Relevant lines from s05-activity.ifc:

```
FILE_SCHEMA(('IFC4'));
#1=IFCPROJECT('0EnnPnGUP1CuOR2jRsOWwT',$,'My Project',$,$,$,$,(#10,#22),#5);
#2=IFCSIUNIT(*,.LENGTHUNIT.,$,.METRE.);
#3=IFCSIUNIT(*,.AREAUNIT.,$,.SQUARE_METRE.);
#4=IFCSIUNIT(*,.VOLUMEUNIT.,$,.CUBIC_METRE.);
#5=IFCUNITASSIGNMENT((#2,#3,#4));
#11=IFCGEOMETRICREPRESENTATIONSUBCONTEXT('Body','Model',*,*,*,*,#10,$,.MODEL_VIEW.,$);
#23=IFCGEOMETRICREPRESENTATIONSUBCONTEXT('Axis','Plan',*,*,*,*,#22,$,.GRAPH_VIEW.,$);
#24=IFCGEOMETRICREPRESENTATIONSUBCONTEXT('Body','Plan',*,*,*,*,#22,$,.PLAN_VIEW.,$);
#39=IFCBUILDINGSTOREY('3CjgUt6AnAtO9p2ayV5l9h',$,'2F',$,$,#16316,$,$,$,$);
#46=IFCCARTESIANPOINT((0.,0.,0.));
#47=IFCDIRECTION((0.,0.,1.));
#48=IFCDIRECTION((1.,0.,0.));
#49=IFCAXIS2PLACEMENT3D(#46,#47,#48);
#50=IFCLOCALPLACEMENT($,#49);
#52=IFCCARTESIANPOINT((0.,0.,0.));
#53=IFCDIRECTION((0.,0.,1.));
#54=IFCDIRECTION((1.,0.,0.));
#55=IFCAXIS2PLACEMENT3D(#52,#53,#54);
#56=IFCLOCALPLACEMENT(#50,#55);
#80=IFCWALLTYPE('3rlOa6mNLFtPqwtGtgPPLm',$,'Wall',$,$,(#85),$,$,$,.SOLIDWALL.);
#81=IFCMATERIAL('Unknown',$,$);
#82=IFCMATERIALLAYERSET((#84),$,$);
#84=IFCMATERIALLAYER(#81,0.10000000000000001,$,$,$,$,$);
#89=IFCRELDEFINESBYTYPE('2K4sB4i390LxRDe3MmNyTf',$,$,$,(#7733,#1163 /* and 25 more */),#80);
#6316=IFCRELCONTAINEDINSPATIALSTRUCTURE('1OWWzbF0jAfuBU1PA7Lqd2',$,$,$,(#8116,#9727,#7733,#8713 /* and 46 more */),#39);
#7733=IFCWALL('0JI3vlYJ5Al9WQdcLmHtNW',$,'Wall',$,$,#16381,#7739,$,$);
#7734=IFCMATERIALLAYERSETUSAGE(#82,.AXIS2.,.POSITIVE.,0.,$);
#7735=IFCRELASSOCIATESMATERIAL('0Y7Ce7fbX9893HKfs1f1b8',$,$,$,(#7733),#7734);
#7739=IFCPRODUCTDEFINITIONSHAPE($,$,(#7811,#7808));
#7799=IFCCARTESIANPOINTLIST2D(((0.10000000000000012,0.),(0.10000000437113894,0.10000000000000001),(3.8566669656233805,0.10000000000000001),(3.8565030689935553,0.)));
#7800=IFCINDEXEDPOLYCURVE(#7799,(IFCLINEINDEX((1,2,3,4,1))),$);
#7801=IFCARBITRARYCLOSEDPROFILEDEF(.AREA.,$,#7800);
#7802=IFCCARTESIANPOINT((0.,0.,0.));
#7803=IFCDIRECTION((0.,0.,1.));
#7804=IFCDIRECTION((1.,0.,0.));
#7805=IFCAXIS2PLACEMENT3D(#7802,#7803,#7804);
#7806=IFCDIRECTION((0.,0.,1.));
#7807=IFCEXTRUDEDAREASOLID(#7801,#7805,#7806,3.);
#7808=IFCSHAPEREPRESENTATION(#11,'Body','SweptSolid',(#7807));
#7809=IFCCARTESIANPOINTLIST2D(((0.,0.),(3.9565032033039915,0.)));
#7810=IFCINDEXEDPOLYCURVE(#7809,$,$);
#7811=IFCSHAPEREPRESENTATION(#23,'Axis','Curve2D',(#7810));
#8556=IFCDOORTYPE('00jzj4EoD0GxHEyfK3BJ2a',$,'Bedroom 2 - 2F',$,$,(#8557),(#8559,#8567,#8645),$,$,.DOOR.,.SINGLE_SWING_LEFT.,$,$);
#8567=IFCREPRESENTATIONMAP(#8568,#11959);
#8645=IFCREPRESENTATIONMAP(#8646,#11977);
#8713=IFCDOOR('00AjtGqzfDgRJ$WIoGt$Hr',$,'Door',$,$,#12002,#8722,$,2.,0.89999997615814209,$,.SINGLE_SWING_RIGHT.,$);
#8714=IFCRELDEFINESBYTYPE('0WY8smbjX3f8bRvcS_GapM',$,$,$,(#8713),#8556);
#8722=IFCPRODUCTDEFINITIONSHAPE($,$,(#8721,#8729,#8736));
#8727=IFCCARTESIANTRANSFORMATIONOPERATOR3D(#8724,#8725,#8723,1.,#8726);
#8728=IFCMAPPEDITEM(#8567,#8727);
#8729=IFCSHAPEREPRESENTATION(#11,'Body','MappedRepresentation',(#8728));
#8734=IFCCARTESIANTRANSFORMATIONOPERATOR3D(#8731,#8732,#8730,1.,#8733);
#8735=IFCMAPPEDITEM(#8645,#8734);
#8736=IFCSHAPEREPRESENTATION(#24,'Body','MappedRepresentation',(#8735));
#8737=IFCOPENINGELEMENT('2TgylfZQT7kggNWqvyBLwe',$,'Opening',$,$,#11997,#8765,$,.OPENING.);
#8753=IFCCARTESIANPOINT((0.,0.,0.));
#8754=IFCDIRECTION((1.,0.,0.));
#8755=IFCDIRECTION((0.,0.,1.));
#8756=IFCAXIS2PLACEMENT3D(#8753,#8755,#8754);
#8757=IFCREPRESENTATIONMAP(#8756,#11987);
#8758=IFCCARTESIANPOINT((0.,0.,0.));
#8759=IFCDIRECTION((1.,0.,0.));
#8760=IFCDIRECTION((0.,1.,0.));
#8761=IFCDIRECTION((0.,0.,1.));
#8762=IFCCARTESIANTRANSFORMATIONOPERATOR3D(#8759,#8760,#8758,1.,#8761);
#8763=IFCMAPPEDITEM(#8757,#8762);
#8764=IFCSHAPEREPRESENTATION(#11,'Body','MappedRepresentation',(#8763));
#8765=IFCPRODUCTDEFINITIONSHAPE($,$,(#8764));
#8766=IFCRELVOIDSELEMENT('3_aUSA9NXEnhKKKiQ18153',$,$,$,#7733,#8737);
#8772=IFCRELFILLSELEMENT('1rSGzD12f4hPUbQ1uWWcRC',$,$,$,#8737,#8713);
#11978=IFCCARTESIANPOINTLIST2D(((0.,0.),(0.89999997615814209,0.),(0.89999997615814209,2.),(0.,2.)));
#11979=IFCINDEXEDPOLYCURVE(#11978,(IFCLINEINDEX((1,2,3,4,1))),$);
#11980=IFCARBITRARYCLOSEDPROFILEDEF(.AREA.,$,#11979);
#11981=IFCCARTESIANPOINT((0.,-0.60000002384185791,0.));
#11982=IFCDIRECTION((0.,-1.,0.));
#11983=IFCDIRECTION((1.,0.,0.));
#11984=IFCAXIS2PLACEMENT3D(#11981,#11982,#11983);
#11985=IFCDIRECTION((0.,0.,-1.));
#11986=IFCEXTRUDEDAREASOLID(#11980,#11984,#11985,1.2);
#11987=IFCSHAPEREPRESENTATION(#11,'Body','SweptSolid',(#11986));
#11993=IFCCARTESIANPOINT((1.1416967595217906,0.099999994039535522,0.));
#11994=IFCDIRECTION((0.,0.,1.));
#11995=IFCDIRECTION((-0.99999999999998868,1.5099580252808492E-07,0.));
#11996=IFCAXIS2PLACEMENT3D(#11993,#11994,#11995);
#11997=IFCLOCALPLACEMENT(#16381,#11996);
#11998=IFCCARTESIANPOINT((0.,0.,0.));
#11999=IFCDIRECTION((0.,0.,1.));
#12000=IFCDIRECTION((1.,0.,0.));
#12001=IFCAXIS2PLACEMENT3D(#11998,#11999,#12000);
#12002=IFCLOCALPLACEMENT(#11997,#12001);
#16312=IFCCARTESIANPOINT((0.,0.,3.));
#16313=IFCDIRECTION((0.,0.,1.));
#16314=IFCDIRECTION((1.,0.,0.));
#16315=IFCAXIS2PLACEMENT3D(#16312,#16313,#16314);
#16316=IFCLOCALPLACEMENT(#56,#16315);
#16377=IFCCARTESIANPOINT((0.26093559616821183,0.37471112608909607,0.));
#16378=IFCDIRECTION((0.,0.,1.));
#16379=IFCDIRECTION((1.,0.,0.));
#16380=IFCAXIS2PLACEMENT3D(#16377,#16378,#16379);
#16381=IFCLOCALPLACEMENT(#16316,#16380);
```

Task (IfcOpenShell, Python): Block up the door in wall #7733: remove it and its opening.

```python
import ifcopenshell
import ifcopenshell.api.feature
import ifcopenshell.api.root
import ifcopenshell.geom
import ifcopenshell.util.shape

model = ifcopenshell.open("s05-activity.ifc")
settings = ifcopenshell.geom.settings()


def volume(element):
    """Net volume in cubic metres, openings subtracted."""
    shape = ifcopenshell.geom.create_shape(settings, element)
    return ifcopenshell.util.shape.get_volume(shape.geometry)


door = model.by_guid("00AjtGqzfDgRJ$WIoGt$Hr")
opening = door.FillsVoids[0].RelatingOpeningElement
wall = opening.VoidsElements[0].RelatingBuildingElement
before = volume(wall)

ifcopenshell.api.root.remove_product(model, product=door)
ifcopenshell.api.feature.remove_feature(model, feature=opening)

after = volume(wall)

print(f"wall volume {before:.3f} -> {after:.3f} m3")

model.write("s05-activity_v2.ifc")
```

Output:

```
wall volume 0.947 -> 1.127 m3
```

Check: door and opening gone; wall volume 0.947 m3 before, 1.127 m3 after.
